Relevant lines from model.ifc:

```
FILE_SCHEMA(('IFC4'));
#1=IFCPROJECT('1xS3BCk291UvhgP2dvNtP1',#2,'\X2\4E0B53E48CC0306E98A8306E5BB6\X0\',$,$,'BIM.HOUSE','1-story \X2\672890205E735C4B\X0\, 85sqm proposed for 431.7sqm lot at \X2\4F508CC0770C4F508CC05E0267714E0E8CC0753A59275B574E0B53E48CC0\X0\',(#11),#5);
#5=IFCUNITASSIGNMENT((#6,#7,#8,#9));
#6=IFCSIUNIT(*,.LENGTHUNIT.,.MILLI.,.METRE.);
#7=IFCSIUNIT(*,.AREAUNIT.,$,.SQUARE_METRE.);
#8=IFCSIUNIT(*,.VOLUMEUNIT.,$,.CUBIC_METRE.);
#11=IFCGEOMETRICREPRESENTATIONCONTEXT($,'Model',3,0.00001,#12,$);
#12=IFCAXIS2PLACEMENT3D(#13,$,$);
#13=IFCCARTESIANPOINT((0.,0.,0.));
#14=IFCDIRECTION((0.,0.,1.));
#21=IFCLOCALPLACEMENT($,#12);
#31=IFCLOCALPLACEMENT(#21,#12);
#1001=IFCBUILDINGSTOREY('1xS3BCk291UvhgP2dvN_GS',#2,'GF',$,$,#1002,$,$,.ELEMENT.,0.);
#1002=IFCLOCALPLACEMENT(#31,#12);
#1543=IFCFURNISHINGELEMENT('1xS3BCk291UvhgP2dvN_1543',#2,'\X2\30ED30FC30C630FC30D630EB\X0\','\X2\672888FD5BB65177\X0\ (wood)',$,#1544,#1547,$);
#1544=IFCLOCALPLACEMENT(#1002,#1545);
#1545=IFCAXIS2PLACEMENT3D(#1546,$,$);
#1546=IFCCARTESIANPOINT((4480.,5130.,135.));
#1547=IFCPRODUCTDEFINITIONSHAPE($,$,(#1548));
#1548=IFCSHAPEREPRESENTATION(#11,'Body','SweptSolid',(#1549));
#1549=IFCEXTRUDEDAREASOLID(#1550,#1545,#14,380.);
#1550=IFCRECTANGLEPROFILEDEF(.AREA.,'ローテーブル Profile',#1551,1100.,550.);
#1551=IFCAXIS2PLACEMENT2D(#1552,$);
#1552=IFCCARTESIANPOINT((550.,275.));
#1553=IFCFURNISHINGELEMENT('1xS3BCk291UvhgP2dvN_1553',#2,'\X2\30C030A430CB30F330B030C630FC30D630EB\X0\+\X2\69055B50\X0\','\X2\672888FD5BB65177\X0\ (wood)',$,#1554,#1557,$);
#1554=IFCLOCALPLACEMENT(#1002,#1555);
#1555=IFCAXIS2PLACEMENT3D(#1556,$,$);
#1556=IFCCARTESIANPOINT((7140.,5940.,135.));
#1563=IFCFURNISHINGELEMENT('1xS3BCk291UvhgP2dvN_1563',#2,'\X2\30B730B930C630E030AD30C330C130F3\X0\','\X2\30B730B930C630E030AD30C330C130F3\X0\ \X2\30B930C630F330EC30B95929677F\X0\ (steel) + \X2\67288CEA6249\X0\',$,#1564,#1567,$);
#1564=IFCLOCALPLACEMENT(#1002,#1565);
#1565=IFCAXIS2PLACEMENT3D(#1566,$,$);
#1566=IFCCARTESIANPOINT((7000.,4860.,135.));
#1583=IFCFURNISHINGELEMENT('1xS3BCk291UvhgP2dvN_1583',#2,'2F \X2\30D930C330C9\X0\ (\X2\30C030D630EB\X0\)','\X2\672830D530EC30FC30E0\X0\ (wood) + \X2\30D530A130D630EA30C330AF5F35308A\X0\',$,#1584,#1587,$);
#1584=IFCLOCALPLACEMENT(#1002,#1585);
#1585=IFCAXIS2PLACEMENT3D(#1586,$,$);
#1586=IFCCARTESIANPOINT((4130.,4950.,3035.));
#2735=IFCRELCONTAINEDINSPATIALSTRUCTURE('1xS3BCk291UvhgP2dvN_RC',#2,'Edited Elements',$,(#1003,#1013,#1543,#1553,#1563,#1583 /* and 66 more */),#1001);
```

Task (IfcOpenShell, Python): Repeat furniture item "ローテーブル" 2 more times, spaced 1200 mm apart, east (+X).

```python
import numpy as np
import ifcopenshell
import ifcopenshell.api.geometry
import ifcopenshell.api.root
import ifcopenshell.util.element
import ifcopenshell.util.placement
import ifcopenshell.util.unit

model = ifcopenshell.open("model.ifc")
unit_scale = ifcopenshell.util.unit.calculate_unit_scale(model)


def reuse_history(source, copy):
    """copy_class also copies each property set's owner history, people and application; keep the originals."""
    for rel in copy.IsDefinedBy:
        if rel.is_a("IfcRelDefinesByProperties") and (history := rel.RelatingPropertyDefinition.OwnerHistory):
            rel.RelatingPropertyDefinition.OwnerHistory = source.OwnerHistory
            ifcopenshell.util.element.remove_deep2(model, history)


source = model.by_id(1543)
base = ifcopenshell.util.placement.get_local_placement(source.ObjectPlacement)
step = np.array([1.0, 0.0, 0.0]) * 1.2 / unit_scale

for i in range(1, 3):
    copy = ifcopenshell.api.root.copy_class(model, product=source)
    copy.Representation = ifcopenshell.util.element.copy_deep(
        model, source.Representation, exclude=["IfcGeometricRepresentationContext", "IfcRepresentationMap"]
    )
    reuse_history(source, copy)
    matrix = base.copy()
    matrix[:3, 3] += i * step
    print("added at", matrix[:3, 3].round(3) + 0.0)
    ifcopenshell.api.geometry.edit_object_placement(model, product=copy, matrix=matrix, is_si=False)

model.write("model-out.ifc")
```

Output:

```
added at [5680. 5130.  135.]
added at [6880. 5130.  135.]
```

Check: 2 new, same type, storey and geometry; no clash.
